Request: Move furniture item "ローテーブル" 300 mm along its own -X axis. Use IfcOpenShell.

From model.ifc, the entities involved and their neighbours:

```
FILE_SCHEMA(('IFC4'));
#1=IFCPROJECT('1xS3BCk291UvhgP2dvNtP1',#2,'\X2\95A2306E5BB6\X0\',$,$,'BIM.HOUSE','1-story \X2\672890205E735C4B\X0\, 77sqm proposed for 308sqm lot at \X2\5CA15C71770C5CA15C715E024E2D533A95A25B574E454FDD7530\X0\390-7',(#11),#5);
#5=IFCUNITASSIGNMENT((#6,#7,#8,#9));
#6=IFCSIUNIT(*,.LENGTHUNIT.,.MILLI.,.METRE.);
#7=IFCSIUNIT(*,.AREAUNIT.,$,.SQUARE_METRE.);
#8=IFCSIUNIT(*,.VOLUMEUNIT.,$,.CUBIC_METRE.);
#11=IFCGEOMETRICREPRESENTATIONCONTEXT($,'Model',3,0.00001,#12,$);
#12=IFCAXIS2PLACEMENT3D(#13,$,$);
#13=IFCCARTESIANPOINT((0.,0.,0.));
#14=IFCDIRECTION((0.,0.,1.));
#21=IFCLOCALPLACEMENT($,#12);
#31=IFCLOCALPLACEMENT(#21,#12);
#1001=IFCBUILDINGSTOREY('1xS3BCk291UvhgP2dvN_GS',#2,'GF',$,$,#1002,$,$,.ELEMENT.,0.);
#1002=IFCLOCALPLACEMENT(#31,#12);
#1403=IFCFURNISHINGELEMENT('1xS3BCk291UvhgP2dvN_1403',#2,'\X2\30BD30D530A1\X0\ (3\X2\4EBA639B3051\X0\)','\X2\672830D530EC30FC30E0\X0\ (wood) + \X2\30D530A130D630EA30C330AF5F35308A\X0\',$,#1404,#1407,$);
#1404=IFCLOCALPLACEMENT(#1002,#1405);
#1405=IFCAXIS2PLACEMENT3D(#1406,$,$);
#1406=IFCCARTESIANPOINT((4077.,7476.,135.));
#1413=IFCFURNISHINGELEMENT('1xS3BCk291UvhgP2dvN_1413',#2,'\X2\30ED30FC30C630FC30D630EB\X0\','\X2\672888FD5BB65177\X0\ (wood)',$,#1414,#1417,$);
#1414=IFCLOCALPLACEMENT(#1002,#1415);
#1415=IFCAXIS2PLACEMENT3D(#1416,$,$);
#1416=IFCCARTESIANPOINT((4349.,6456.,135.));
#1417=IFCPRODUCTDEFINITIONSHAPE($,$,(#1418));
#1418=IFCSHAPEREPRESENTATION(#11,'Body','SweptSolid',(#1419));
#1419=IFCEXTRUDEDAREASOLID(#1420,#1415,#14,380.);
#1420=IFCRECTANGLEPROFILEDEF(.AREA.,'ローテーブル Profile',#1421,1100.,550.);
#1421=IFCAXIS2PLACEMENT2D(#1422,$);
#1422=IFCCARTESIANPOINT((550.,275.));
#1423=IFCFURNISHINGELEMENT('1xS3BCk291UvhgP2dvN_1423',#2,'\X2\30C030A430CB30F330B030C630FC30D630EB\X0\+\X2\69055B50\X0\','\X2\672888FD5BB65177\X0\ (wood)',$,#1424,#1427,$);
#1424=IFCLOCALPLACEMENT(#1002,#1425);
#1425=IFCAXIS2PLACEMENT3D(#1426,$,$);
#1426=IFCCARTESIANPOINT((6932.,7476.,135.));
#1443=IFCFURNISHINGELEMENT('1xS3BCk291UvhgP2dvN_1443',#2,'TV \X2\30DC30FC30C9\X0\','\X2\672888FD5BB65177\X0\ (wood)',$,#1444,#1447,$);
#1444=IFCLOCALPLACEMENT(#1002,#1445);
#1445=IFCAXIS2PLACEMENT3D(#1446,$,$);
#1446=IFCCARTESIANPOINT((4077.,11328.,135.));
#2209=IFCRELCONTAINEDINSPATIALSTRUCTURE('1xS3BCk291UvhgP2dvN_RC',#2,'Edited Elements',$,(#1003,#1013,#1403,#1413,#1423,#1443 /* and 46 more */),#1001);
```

```python
import ifcopenshell
import ifcopenshell.api.geometry
import ifcopenshell.util.placement

model = ifcopenshell.open("model.ifc")

item = model.by_guid("1xS3BCk291UvhgP2dvN_1413")
matrix = ifcopenshell.util.placement.get_local_placement(item.ObjectPlacement)
matrix[:3, 3] -= matrix[:3, 0] * 300.0
ifcopenshell.api.geometry.edit_object_placement(model, product=item, matrix=matrix, is_si=False)

print(ifcopenshell.util.placement.get_local_placement(item.ObjectPlacement).round(3) + 0.0)

model.write("model_edited.ifc")
```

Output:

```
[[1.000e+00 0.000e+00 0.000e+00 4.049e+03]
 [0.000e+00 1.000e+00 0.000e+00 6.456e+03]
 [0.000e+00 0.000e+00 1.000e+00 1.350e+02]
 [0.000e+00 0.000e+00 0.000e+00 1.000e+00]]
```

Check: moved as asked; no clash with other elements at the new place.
